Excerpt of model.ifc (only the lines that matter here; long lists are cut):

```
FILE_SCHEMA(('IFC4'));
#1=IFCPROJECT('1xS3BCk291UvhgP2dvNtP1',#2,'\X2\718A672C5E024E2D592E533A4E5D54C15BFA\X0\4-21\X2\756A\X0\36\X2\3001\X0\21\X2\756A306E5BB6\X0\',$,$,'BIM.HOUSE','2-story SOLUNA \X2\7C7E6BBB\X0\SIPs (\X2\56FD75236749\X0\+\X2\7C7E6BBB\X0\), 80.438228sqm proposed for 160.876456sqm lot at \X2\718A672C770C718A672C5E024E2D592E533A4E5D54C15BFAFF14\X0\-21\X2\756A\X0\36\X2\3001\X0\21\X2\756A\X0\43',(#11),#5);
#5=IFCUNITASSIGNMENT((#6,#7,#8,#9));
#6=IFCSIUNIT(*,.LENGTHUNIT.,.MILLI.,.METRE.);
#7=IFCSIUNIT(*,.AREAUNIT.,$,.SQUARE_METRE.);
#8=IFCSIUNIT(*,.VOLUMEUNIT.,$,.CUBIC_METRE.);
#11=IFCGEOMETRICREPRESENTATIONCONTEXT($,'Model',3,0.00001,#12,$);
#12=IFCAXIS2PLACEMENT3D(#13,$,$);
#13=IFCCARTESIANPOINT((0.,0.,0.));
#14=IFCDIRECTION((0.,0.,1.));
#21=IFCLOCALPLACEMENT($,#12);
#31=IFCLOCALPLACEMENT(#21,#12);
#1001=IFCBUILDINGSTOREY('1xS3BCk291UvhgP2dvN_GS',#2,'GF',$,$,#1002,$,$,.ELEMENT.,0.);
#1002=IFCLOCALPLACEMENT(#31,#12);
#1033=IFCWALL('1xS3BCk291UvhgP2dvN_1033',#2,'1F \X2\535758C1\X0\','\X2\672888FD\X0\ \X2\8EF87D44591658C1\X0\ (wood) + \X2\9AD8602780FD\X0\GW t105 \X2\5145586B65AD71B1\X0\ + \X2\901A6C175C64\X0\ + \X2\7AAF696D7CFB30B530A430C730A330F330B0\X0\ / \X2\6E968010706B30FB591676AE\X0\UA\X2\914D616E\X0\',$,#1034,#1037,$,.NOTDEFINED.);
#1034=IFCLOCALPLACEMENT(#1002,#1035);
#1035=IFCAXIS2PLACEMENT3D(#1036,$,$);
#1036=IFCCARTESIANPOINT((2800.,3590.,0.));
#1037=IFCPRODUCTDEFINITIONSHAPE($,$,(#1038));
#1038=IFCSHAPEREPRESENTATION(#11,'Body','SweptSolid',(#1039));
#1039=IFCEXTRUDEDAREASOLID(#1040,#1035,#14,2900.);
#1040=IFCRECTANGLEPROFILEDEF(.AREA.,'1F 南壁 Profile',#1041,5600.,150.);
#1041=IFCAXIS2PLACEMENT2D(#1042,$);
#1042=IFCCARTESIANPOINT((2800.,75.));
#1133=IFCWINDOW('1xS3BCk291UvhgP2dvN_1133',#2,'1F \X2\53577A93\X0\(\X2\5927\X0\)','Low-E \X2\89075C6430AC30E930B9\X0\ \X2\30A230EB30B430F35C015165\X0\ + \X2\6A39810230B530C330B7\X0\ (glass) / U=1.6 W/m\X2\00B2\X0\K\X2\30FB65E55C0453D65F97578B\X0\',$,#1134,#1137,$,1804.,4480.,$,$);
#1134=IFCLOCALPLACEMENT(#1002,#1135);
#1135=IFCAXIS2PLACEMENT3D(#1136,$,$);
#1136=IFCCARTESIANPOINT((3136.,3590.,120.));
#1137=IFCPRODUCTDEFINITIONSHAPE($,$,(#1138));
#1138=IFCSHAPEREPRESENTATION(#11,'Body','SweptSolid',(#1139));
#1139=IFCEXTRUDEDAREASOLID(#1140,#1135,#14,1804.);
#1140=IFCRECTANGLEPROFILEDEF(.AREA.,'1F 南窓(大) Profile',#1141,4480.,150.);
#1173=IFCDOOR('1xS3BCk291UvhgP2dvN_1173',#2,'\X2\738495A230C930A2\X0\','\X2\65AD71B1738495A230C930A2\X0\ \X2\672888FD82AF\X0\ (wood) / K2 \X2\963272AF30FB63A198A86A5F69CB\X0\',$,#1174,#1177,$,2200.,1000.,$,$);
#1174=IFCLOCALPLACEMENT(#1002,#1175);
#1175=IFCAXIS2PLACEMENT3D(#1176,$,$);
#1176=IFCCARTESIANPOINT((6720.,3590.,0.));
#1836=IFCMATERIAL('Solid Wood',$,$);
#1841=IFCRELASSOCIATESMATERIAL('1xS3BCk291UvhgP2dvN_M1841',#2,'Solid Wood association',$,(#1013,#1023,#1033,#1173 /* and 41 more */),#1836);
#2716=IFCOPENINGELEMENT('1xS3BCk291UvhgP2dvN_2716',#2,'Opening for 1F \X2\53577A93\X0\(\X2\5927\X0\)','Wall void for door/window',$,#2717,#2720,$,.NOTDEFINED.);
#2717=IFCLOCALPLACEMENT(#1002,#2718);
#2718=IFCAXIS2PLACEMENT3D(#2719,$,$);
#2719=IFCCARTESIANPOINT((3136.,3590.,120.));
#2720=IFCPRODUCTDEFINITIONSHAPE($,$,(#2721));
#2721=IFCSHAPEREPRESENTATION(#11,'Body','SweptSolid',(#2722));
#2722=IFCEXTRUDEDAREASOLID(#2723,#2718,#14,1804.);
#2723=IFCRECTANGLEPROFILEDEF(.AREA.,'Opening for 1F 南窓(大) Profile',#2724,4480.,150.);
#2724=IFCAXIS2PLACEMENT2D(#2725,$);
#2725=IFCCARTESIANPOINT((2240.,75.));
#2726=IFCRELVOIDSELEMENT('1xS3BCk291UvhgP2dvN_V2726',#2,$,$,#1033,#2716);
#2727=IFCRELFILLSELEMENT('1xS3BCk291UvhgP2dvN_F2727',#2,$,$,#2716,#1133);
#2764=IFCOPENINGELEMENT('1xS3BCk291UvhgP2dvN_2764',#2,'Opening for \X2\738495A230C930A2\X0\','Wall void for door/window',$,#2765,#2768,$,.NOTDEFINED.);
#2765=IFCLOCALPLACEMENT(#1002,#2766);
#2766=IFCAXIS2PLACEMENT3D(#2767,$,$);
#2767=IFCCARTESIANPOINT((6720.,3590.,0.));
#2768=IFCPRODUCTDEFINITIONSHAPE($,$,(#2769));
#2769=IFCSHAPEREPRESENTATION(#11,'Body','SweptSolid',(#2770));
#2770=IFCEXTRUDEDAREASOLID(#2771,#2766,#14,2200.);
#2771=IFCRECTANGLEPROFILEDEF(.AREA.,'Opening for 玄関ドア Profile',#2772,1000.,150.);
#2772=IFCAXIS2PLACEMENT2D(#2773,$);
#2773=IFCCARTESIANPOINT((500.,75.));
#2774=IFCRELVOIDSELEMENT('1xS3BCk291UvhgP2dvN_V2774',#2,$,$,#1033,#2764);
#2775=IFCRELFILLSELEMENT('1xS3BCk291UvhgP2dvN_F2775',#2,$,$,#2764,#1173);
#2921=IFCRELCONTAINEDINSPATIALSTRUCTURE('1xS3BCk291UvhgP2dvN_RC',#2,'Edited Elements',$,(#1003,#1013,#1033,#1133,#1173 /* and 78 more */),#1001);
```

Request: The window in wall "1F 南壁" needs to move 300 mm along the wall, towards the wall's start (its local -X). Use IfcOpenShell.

```python
import ifcopenshell
import ifcopenshell.api.geometry
import ifcopenshell.util.placement
import ifcopenshell.util.unit

model = ifcopenshell.open("model.ifc")
unit_scale = ifcopenshell.util.unit.calculate_unit_scale(model)

window = model.by_guid("1xS3BCk291UvhgP2dvN_1133")
opening = window.FillsVoids[0].RelatingOpeningElement
wall = opening.VoidsElements[0].RelatingBuildingElement

wall_matrix = ifcopenshell.util.placement.get_local_placement(wall.ObjectPlacement)
shift = wall_matrix[:3, 0] * -0.3 / unit_scale
before = ifcopenshell.util.placement.get_local_placement(window.ObjectPlacement)[:3, 3].copy()

# The window is not placed relative to its opening, so move both.
for product in (opening, window):
    matrix = ifcopenshell.util.placement.get_local_placement(product.ObjectPlacement)
    matrix[:3, 3] += shift
    ifcopenshell.api.geometry.edit_object_placement(model, product=product, matrix=matrix, is_si=False)

after = ifcopenshell.util.placement.get_local_placement(window.ObjectPlacement)[:3, 3]
print("window moved by", (after - before).round(3) + 0.0)

model.write("model_v2.ifc")
```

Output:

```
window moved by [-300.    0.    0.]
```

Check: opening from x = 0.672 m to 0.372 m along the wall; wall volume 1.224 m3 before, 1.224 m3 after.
